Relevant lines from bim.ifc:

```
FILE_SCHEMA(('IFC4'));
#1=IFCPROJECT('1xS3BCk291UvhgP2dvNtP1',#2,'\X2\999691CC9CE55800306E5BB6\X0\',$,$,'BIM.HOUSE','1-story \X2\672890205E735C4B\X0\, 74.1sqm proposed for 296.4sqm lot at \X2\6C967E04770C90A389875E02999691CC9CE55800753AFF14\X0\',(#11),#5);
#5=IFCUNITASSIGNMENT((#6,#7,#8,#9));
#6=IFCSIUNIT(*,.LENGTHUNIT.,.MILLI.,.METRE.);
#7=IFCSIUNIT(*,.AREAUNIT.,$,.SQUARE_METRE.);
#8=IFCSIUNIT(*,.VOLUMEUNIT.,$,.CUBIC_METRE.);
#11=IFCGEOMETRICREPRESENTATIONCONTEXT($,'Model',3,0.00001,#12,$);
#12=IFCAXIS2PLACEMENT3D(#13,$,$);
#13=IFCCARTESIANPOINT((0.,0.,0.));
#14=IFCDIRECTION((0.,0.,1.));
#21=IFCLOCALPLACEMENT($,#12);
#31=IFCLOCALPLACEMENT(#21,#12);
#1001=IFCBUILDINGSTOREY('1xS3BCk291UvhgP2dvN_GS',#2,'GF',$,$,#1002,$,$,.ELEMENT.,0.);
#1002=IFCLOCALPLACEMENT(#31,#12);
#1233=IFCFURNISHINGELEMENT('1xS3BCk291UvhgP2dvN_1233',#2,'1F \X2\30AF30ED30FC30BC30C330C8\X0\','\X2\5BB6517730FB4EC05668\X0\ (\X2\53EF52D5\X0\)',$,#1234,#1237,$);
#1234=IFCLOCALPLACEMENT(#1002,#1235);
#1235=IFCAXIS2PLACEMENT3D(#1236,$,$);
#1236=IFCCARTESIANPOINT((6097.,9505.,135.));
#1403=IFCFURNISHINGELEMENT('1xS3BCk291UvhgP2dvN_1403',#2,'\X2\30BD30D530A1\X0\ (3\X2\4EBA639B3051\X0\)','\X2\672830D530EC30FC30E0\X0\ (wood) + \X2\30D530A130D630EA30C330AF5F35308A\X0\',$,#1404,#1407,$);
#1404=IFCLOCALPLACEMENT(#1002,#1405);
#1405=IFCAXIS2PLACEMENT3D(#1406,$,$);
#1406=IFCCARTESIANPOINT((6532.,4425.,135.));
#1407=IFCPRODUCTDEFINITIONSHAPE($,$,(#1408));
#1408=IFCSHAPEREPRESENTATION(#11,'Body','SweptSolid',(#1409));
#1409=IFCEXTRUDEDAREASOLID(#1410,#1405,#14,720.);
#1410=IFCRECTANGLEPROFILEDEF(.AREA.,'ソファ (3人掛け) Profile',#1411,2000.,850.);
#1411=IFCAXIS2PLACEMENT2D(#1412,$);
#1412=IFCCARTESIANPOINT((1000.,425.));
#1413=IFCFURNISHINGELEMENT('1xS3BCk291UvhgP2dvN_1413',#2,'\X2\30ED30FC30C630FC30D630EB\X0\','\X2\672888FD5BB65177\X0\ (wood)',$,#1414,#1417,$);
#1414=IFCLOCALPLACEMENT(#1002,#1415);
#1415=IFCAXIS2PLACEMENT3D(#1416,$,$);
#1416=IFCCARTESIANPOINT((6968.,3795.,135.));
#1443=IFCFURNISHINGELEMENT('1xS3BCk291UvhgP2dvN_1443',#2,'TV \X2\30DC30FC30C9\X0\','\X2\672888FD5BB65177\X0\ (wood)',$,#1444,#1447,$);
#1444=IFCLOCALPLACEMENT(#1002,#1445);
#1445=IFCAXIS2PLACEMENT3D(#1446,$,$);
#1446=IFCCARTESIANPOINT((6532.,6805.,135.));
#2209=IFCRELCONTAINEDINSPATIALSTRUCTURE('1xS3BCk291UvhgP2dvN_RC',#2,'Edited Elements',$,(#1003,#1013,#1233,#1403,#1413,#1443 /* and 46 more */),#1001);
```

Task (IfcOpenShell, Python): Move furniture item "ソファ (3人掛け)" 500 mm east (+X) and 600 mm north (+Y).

```python
import ifcopenshell
import ifcopenshell.api.geometry
import ifcopenshell.util.placement
import ifcopenshell.util.unit

model = ifcopenshell.open("bim.ifc")
unit_scale = ifcopenshell.util.unit.calculate_unit_scale(model)

item = model.by_guid("1xS3BCk291UvhgP2dvN_1403")
matrix = ifcopenshell.util.placement.get_local_placement(item.ObjectPlacement)
matrix[0, 3] += 0.5 / unit_scale
matrix[1, 3] += 0.6 / unit_scale
ifcopenshell.api.geometry.edit_object_placement(model, product=item, matrix=matrix, is_si=False)

print(ifcopenshell.util.placement.get_local_placement(item.ObjectPlacement).round(3) + 0.0)

model.write("bim_updated.ifc")
```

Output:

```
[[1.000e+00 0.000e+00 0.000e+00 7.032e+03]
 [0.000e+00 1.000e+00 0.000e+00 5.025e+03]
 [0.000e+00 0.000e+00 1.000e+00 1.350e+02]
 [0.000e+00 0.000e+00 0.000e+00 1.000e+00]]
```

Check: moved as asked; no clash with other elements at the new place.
